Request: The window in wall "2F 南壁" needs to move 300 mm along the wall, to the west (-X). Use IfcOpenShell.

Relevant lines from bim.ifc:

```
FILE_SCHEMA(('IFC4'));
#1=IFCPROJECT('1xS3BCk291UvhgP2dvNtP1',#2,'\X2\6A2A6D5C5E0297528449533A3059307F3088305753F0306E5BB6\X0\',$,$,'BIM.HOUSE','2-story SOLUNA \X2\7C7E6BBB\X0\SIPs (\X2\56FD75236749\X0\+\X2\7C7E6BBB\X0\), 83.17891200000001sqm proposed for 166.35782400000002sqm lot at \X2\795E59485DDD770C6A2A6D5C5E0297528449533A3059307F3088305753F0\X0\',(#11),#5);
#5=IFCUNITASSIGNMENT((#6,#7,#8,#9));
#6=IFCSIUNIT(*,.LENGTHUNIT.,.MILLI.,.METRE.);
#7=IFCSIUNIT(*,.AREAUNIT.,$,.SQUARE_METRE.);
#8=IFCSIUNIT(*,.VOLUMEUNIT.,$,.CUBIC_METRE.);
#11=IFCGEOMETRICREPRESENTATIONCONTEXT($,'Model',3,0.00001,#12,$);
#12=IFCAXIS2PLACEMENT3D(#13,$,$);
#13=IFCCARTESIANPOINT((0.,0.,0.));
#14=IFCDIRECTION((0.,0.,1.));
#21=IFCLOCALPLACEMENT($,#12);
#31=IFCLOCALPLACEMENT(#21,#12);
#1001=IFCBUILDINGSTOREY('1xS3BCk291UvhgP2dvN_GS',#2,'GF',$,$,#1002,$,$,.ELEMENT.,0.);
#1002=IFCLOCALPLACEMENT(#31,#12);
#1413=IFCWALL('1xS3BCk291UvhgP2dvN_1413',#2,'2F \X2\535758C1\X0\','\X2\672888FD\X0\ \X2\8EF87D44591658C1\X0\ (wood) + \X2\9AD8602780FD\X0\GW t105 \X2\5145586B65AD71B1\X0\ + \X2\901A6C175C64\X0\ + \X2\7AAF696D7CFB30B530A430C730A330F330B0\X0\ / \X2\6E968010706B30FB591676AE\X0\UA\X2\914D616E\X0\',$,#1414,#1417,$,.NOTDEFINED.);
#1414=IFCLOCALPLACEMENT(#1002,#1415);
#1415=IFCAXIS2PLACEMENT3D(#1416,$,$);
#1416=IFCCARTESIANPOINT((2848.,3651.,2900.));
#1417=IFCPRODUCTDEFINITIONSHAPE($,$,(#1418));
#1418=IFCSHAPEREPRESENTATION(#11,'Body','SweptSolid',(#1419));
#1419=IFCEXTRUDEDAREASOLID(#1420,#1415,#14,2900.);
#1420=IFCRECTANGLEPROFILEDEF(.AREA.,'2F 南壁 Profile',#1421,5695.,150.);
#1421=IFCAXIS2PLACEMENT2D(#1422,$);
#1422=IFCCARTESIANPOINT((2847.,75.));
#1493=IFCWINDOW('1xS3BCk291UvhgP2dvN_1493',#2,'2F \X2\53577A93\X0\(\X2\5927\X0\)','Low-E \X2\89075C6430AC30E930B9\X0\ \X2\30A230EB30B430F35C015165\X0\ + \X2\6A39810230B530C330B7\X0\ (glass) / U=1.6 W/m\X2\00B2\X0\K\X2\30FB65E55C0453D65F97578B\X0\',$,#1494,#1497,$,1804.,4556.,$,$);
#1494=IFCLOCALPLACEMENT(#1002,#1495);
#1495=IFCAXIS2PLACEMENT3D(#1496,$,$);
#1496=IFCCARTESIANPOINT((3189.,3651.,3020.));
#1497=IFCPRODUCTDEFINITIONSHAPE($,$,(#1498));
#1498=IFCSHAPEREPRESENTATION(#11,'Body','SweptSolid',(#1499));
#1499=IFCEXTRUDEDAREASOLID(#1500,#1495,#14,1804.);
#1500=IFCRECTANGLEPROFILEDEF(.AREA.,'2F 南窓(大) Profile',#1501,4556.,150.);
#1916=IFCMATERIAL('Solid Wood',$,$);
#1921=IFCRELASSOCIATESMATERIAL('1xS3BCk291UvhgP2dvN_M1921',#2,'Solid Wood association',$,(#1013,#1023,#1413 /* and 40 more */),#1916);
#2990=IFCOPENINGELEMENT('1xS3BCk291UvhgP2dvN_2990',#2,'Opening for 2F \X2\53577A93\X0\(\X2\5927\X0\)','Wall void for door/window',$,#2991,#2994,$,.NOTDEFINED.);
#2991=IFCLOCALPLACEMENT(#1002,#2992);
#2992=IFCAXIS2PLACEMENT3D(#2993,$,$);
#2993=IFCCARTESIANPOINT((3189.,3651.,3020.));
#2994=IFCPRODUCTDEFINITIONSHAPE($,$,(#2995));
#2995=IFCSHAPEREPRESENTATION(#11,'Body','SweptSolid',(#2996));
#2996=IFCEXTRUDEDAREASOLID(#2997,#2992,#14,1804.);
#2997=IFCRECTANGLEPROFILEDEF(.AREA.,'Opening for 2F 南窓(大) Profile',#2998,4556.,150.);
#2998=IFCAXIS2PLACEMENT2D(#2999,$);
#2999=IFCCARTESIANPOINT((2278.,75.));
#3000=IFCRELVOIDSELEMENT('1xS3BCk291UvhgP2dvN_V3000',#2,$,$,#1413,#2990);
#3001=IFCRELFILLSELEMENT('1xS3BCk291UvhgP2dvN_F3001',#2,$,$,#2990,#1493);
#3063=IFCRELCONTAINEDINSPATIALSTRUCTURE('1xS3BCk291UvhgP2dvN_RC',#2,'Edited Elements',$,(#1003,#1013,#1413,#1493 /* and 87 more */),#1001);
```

```python
import ifcopenshell
import ifcopenshell.api.geometry
import ifcopenshell.util.placement
import ifcopenshell.util.unit

model = ifcopenshell.open("bim.ifc")
unit_scale = ifcopenshell.util.unit.calculate_unit_scale(model)

window = model.by_guid("1xS3BCk291UvhgP2dvN_1493")
opening = window.FillsVoids[0].RelatingOpeningElement
wall = opening.VoidsElements[0].RelatingBuildingElement

wall_matrix = ifcopenshell.util.placement.get_local_placement(wall.ObjectPlacement)
shift = wall_matrix[:3, 0] * -0.3 / unit_scale
before = ifcopenshell.util.placement.get_local_placement(window.ObjectPlacement)[:3, 3].copy()

# The window is not placed relative to its opening, so move both.
for product in (opening, window):
    matrix = ifcopenshell.util.placement.get_local_placement(product.ObjectPlacement)
    matrix[:3, 3] += shift
    ifcopenshell.api.geometry.edit_object_placement(model, product=product, matrix=matrix, is_si=False)

after = ifcopenshell.util.placement.get_local_placement(window.ObjectPlacement)[:3, 3]
print("window moved by", (after - before).round(3) + 0.0)

model.write("bim_v2.ifc")
```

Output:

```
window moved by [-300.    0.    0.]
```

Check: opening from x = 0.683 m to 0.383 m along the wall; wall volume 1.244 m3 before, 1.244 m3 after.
